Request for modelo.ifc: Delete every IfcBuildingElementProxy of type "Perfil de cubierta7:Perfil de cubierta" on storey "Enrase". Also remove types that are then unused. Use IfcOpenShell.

First a look at what the model holds.

```python
import ifcopenshell
import ifcopenshell.util.element

model = ifcopenshell.open("modelo.ifc")
print(model.schema)
storey = next(s for s in model.by_type("IfcBuildingStorey") if s.Name == "Enrase")
proxies = [e for e in ifcopenshell.util.element.get_decomposition(storey) if e.is_a("IfcBuildingElementProxy")]
seen = {}
for e in proxies:
    element_type = ifcopenshell.util.element.get_type(e)
    name = element_type.Name if element_type not in (None, e) else None
    seen[name] = seen.get(name, 0) + 1
for name, count in sorted(seen.items(), key=str):
    print(count, "x", name)
```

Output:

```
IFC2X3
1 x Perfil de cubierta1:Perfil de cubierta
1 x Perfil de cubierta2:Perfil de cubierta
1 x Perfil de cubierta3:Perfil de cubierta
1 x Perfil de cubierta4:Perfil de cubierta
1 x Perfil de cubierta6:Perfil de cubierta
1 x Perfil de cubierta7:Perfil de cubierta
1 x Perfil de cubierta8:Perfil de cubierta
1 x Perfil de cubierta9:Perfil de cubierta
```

```python
import ifcopenshell
import ifcopenshell.api.root
import ifcopenshell.util.element

model = ifcopenshell.open("modelo.ifc")

storey = next(s for s in model.by_type("IfcBuildingStorey") if s.Name == "Enrase")
proxies = [e for e in ifcopenshell.util.element.get_decomposition(storey) if e.is_a("IfcBuildingElementProxy")]
targets = [e for e in proxies if (t := ifcopenshell.util.element.get_type(e)) not in (None, e) and t.Name == "Perfil de cubierta7:Perfil de cubierta"]
types = {ifcopenshell.util.element.get_type(e) for e in targets} - {None, *targets}

for e in targets:
    ifcopenshell.api.root.remove_product(model, product=e)
print(len(targets), "removed")

unused = [t for t in types if not ifcopenshell.util.element.get_types(t)]
for t in unused:
    ifcopenshell.api.root.remove_product(model, product=t)
print(len(unused), "unused types removed")

model.write("modelo_v2.ifc")
```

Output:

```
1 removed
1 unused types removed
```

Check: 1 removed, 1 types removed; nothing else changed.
